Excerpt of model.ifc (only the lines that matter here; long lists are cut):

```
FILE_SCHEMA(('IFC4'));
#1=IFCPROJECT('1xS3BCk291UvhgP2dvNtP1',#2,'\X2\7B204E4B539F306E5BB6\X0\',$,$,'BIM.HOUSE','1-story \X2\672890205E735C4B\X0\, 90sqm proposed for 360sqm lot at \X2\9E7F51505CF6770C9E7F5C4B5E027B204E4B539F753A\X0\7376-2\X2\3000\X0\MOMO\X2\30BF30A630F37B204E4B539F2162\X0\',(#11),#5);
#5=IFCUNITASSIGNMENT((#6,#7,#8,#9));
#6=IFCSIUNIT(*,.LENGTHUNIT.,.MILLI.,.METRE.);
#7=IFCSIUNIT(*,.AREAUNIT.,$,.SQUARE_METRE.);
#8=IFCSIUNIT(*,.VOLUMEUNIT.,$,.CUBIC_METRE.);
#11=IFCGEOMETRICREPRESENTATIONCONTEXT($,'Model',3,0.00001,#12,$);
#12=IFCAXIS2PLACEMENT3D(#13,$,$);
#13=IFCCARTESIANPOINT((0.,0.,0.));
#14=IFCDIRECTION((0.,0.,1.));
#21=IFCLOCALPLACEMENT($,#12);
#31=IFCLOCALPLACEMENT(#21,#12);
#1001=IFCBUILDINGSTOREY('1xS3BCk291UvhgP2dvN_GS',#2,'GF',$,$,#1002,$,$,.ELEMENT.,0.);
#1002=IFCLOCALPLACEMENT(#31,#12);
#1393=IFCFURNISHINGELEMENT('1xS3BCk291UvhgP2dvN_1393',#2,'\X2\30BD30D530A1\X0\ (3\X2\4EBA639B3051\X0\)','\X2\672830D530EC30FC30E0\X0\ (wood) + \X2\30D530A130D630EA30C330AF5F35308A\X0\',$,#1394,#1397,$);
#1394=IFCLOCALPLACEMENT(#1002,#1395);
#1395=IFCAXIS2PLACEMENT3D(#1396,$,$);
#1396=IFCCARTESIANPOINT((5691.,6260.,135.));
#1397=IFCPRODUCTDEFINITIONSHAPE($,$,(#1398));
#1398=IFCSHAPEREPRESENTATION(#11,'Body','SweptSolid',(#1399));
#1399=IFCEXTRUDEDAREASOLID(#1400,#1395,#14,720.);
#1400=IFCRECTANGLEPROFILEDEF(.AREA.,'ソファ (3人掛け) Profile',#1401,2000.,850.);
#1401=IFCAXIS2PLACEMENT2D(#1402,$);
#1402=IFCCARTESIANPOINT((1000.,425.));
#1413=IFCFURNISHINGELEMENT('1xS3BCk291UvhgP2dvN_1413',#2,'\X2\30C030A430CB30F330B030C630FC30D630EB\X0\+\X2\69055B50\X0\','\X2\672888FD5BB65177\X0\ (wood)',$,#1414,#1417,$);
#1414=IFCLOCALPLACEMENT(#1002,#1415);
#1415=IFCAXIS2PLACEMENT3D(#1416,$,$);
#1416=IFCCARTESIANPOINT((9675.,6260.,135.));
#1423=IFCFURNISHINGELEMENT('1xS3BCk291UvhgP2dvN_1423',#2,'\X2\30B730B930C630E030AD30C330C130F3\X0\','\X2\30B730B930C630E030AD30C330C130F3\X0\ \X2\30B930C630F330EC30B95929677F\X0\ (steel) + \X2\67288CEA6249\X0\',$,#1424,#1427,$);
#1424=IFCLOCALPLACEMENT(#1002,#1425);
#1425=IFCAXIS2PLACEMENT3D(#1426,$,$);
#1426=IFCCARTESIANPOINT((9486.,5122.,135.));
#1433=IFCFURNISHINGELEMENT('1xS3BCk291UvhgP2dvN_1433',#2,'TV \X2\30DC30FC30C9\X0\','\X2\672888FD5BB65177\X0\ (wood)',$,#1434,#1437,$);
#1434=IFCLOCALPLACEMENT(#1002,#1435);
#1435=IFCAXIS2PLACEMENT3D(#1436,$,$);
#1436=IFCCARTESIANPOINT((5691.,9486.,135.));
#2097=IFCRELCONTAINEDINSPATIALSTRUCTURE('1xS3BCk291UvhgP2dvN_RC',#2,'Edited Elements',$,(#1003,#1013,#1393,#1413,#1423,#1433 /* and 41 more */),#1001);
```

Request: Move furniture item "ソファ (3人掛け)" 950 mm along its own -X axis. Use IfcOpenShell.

```python
import ifcopenshell
import ifcopenshell.api.geometry
import ifcopenshell.util.placement
import ifcopenshell.util.unit

model = ifcopenshell.open("model.ifc")
unit_scale = ifcopenshell.util.unit.calculate_unit_scale(model)

item = model.by_id(1393)
matrix = ifcopenshell.util.placement.get_local_placement(item.ObjectPlacement)
matrix[:3, 3] -= matrix[:3, 0] * 0.95 / unit_scale
ifcopenshell.api.geometry.edit_object_placement(model, product=item, matrix=matrix, is_si=False)

print(ifcopenshell.util.placement.get_local_placement(item.ObjectPlacement).round(3) + 0.0)

model.write("model_v2.ifc")
```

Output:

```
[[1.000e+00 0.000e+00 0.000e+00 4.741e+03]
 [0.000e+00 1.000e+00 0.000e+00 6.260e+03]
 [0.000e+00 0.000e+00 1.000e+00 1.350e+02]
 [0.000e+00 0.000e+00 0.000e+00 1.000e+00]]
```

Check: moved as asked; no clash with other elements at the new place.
